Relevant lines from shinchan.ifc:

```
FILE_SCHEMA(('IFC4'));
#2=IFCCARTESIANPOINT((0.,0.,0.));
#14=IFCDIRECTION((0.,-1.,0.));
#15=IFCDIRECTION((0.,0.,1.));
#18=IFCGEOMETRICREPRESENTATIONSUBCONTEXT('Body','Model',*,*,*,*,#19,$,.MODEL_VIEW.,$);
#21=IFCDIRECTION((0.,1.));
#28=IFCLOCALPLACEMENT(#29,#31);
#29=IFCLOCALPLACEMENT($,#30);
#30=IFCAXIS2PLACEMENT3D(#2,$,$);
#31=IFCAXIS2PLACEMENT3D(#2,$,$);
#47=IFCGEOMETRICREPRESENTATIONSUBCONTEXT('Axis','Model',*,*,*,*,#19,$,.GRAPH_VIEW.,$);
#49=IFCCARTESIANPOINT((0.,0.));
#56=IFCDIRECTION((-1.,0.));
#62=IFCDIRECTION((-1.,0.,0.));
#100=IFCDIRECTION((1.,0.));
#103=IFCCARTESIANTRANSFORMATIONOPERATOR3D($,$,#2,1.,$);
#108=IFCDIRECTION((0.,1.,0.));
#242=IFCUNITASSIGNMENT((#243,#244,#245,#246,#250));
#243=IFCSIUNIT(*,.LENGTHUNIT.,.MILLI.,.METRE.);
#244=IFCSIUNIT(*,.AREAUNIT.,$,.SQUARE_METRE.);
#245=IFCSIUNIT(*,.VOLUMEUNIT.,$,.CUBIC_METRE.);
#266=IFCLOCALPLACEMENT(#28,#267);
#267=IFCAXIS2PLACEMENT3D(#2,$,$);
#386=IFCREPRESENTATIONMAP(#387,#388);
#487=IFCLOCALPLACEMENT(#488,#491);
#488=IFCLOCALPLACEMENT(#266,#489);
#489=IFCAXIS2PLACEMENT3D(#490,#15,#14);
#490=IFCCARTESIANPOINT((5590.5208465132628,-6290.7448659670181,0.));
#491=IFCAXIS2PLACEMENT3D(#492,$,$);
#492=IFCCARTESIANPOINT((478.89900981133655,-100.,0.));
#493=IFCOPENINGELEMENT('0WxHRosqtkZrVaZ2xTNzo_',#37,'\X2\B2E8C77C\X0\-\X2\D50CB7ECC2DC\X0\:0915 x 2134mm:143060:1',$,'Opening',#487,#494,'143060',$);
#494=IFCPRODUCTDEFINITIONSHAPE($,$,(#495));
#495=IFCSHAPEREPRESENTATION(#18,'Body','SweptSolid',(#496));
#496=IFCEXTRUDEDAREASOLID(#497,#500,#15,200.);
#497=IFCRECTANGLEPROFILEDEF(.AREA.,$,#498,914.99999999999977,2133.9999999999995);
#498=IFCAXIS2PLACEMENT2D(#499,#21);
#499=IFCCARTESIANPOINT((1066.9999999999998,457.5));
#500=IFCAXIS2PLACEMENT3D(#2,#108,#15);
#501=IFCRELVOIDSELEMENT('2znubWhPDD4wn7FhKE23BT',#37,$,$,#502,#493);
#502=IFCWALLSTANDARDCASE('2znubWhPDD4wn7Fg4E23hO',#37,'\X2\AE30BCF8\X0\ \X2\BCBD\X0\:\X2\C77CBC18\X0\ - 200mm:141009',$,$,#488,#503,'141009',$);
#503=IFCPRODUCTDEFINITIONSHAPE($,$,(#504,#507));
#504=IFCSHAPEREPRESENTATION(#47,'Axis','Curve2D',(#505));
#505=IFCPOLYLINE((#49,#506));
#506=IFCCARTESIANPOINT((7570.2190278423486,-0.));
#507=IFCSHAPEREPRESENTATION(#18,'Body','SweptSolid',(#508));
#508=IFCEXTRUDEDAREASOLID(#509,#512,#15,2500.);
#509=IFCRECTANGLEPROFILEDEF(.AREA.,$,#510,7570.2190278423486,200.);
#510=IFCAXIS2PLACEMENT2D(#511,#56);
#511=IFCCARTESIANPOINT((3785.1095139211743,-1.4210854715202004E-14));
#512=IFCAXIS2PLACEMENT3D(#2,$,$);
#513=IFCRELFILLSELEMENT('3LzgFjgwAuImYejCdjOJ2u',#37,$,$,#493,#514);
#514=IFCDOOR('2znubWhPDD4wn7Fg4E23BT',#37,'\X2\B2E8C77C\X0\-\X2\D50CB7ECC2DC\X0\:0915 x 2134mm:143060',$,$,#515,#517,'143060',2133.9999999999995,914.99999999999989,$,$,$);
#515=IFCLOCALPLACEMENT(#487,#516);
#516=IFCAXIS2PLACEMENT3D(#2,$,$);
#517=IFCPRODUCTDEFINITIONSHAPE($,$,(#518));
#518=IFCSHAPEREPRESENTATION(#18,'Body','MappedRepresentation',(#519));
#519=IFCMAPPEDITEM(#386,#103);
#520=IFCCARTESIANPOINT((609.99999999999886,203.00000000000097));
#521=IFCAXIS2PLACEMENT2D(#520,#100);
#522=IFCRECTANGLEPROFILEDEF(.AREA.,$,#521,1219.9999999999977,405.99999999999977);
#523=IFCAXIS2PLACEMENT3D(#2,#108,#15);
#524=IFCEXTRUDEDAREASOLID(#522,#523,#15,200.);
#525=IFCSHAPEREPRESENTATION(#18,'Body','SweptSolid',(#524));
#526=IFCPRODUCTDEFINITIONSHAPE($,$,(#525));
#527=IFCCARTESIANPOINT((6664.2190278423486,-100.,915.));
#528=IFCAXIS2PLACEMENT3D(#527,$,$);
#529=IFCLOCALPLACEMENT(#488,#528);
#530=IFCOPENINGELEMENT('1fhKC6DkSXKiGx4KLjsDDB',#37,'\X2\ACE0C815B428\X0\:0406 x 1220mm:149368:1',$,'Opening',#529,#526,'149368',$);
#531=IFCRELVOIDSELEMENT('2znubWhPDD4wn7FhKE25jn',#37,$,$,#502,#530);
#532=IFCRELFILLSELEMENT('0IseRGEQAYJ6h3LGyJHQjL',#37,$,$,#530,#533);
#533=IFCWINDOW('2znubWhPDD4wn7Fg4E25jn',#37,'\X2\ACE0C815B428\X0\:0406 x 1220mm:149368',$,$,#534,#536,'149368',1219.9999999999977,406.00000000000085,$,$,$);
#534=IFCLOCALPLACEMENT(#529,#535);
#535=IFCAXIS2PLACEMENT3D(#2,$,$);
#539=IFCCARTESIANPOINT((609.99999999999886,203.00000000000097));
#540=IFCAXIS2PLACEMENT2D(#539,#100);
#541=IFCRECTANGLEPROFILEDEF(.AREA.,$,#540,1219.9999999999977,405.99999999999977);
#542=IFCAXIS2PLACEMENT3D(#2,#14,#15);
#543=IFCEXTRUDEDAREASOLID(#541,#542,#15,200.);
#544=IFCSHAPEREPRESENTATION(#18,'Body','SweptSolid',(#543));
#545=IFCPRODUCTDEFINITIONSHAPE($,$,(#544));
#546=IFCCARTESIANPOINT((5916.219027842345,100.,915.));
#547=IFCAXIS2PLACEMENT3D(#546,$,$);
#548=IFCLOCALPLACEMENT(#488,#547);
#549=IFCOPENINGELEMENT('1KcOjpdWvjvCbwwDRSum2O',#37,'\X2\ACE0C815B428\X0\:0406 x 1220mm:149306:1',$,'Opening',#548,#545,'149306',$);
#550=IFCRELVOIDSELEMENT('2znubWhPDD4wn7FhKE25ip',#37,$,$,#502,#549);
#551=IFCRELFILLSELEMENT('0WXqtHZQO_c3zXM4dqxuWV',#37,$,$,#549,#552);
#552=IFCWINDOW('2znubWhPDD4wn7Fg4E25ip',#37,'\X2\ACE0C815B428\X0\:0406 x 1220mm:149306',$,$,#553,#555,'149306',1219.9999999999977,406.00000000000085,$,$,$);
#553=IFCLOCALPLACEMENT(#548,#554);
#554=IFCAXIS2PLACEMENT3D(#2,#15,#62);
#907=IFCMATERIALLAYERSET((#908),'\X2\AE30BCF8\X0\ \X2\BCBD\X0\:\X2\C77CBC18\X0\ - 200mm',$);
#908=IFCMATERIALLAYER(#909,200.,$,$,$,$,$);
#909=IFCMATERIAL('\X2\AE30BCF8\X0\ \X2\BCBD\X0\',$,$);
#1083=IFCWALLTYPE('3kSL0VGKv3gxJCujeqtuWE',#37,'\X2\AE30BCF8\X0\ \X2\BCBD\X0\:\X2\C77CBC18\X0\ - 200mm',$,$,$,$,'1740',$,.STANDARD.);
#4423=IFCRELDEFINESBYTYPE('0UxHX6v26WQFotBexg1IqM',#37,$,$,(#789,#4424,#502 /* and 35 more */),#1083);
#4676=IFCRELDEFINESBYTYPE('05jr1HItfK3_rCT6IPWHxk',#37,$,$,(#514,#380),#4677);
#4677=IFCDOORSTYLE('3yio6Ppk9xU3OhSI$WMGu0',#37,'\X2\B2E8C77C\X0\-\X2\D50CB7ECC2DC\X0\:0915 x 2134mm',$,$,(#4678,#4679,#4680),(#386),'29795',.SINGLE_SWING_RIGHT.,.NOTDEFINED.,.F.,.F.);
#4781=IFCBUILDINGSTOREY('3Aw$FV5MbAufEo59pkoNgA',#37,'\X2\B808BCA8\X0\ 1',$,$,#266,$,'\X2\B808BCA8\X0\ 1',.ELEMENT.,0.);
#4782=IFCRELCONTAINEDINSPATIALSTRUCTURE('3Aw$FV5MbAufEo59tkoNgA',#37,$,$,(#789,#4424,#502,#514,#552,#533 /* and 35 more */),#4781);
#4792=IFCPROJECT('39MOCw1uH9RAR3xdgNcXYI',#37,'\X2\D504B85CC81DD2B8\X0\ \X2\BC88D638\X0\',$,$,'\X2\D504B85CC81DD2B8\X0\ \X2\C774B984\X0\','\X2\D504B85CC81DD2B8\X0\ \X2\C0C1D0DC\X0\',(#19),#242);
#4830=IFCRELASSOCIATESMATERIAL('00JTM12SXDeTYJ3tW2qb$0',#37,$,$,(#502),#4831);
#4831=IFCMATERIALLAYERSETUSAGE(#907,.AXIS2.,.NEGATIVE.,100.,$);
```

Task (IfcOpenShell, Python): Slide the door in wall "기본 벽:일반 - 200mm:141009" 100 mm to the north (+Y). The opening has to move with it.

```python
import ifcopenshell
import ifcopenshell.api.geometry
import ifcopenshell.util.placement

model = ifcopenshell.open("shinchan.ifc")

door = model.by_guid("2znubWhPDD4wn7Fg4E23BT")
opening = door.FillsVoids[0].RelatingOpeningElement
wall = opening.VoidsElements[0].RelatingBuildingElement

wall_matrix = ifcopenshell.util.placement.get_local_placement(wall.ObjectPlacement)
shift = wall_matrix[:3, 0] * -100.0
before = ifcopenshell.util.placement.get_local_placement(door.ObjectPlacement)[:3, 3].copy()

# The door is placed relative to its opening, so it follows when the opening moves.
matrix = ifcopenshell.util.placement.get_local_placement(opening.ObjectPlacement)
matrix[:3, 3] += shift
ifcopenshell.api.geometry.edit_object_placement(
    model, product=opening, matrix=matrix, is_si=False, should_transform_children=True
)

after = ifcopenshell.util.placement.get_local_placement(door.ObjectPlacement)[:3, 3]
print("door moved by", (after - before).round(3) + 0.0)

model.write("shinchan-out.ifc")
```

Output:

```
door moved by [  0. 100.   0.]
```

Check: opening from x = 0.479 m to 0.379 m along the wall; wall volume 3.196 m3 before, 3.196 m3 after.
